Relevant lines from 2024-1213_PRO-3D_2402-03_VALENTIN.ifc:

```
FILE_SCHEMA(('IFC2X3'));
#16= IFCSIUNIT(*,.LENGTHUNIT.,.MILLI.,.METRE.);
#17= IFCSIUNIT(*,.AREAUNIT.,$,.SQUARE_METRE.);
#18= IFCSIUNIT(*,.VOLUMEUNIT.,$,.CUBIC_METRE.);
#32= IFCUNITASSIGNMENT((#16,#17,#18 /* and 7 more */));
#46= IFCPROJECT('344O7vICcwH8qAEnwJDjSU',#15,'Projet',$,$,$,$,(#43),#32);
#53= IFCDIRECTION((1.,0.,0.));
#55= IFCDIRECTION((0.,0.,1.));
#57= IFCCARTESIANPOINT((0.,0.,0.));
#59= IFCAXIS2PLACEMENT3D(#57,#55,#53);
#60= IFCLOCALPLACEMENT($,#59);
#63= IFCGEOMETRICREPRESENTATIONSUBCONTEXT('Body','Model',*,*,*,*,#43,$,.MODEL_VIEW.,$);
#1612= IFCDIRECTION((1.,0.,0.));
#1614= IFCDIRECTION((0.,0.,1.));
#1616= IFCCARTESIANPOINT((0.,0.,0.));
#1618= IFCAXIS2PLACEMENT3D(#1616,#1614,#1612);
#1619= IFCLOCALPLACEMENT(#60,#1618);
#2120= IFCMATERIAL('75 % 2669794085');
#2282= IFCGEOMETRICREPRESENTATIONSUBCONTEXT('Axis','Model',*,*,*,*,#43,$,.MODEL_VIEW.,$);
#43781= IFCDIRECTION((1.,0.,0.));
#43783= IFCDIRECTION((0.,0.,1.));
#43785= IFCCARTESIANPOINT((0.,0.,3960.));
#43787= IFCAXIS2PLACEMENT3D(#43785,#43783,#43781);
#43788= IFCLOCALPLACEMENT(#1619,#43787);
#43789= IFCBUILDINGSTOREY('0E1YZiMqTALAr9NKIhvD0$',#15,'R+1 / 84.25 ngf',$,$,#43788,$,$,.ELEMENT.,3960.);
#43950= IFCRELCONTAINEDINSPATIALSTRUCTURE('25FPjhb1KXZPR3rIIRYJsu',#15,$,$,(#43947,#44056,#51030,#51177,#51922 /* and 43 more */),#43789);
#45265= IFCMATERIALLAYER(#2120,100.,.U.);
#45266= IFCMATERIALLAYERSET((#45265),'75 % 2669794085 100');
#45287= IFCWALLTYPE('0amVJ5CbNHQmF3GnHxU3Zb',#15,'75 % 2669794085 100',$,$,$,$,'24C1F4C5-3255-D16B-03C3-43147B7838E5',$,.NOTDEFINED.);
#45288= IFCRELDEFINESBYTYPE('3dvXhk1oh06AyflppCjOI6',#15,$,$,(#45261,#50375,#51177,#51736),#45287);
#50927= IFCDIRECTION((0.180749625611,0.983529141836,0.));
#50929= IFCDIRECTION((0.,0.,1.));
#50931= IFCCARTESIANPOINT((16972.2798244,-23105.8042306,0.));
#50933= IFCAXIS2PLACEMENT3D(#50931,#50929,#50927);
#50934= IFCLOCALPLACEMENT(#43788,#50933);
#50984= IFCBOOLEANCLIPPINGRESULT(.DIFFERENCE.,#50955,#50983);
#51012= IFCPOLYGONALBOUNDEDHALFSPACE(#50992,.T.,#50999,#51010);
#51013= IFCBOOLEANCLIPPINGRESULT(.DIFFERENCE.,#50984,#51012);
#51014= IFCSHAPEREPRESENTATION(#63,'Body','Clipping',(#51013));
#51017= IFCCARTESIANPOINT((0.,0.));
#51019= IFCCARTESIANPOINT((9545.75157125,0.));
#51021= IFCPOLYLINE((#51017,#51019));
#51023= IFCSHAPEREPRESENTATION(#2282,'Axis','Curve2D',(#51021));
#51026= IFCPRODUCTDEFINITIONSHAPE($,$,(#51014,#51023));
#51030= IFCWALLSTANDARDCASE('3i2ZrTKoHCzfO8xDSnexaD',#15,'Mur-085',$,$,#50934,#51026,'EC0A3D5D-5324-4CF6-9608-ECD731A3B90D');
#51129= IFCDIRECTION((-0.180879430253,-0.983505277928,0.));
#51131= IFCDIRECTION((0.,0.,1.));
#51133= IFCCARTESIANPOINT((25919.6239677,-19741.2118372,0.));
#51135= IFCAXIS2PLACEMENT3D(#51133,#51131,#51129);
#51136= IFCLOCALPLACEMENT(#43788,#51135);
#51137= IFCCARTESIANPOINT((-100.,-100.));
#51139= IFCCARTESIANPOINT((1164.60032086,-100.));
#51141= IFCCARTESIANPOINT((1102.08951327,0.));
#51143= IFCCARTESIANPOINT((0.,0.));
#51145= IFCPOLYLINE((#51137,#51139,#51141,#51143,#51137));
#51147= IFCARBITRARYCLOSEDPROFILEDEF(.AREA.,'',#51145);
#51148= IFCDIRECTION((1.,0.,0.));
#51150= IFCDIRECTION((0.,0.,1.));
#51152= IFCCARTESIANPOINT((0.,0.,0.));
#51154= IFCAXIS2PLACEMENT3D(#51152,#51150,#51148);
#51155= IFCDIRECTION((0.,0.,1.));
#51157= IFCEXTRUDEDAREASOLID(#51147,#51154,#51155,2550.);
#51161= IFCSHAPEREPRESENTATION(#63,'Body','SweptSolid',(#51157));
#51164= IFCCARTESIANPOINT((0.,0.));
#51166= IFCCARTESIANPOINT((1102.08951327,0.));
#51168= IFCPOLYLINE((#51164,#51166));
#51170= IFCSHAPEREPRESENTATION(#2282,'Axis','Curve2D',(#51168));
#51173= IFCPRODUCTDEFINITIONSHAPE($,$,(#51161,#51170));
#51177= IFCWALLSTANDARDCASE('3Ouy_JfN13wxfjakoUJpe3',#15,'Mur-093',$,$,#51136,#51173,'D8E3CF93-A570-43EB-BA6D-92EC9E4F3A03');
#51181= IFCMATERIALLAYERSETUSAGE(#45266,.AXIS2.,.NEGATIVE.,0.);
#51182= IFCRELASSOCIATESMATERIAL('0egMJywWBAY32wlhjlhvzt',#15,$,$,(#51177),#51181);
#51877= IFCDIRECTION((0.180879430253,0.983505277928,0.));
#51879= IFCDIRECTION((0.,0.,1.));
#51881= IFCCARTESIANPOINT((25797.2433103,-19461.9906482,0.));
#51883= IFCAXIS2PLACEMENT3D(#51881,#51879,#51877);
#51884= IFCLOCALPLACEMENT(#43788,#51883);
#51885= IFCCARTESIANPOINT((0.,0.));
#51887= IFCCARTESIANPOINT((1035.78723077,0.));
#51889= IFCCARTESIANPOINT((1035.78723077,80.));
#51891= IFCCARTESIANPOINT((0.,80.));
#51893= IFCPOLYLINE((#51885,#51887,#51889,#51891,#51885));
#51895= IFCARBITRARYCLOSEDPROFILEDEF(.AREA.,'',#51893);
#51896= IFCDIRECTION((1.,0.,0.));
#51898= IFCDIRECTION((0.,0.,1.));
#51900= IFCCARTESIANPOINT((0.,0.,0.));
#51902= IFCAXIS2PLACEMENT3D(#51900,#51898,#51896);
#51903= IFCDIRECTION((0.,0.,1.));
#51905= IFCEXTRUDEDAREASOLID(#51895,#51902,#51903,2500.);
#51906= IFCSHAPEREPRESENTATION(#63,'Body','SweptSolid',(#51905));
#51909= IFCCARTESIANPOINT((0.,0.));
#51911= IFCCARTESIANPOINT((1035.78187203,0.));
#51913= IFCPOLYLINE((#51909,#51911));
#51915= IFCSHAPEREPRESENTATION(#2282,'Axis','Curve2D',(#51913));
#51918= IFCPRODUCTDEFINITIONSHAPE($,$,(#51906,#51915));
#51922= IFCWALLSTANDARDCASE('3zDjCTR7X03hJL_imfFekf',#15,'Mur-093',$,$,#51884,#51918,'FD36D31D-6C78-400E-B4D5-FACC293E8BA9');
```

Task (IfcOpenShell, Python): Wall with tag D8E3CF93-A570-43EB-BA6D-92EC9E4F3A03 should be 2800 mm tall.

```python
import ifcopenshell
import ifcopenshell.geom
import ifcopenshell.util.representation
import ifcopenshell.util.shape

model = ifcopenshell.open("2024-1213_PRO-3D_2402-03_VALENTIN.ifc")
settings = ifcopenshell.geom.settings()


def volume(element):
    """Net volume in cubic metres, openings subtracted."""
    shape = ifcopenshell.geom.create_shape(settings, element)
    return ifcopenshell.util.shape.get_volume(shape.geometry)


wall = model.by_id(51177)
before = volume(wall)

body = ifcopenshell.util.representation.get_representation(wall, "Model", "Body")
solid = body.Items[0]
old_height = solid.Depth
solid.Depth = 2800.0
after = volume(wall)

print(f"height {old_height:g} -> {solid.Depth:g}, volume {before:.3f} -> {after:.3f} m3")

model.write("2024-1213_PRO-3D_2402-03_VALENTIN_v2.ifc")
```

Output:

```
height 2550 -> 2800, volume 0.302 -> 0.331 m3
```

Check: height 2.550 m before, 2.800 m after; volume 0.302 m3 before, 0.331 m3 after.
